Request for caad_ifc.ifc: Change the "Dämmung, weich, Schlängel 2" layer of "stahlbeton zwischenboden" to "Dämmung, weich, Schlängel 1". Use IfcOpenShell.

First a look at what the model holds.

```python
import ifcopenshell
import ifcopenshell.util.element

model = ifcopenshell.open("caad_ifc.ifc")
print(model.schema)
for layer_set in model.by_type("IfcMaterialLayerSet"):
    if layer_set.LayerSetName == "stahlbeton zwischenboden":
        for layer in layer_set.MaterialLayers:
            print(layer.id(), layer.Material and layer.Material.Name, layer.LayerThickness, sep=" | ")
        print(len(ifcopenshell.util.element.get_elements_by_material(model, layer_set)), "elements and types use it")
print(sorted(m.Name for m in model.by_type("IfcMaterial") if m.Name)[:60])
```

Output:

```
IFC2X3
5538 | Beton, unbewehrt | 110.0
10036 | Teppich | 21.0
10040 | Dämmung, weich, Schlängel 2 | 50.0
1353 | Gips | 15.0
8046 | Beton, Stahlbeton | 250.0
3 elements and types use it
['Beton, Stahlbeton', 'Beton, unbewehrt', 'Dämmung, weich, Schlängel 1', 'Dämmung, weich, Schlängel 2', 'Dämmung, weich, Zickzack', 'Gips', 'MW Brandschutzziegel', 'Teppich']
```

```python
import ifcopenshell
import ifcopenshell.api.material

model = ifcopenshell.open("caad_ifc.ifc")

layer_set = next(s for s in model.by_type("IfcMaterialLayerSet") if s.LayerSetName == "stahlbeton zwischenboden")
layer = next(l for l in layer_set.MaterialLayers if l.Material and l.Material.Name == "Dämmung, weich, Schlängel 2")
material = next(m for m in model.by_type("IfcMaterial") if m.Name == "Dämmung, weich, Schlängel 1")

# Point this one layer at the other material; renaming the old one would change it everywhere.
ifcopenshell.api.material.edit_layer(model, layer=layer, attributes={}, material=material)

print([l.Material.Name if l.Material else None for l in layer_set.MaterialLayers])

model.write("caad_ifc_rev.ifc")
```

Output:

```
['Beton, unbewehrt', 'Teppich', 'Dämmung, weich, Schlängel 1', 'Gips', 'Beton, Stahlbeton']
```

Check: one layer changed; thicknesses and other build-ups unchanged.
